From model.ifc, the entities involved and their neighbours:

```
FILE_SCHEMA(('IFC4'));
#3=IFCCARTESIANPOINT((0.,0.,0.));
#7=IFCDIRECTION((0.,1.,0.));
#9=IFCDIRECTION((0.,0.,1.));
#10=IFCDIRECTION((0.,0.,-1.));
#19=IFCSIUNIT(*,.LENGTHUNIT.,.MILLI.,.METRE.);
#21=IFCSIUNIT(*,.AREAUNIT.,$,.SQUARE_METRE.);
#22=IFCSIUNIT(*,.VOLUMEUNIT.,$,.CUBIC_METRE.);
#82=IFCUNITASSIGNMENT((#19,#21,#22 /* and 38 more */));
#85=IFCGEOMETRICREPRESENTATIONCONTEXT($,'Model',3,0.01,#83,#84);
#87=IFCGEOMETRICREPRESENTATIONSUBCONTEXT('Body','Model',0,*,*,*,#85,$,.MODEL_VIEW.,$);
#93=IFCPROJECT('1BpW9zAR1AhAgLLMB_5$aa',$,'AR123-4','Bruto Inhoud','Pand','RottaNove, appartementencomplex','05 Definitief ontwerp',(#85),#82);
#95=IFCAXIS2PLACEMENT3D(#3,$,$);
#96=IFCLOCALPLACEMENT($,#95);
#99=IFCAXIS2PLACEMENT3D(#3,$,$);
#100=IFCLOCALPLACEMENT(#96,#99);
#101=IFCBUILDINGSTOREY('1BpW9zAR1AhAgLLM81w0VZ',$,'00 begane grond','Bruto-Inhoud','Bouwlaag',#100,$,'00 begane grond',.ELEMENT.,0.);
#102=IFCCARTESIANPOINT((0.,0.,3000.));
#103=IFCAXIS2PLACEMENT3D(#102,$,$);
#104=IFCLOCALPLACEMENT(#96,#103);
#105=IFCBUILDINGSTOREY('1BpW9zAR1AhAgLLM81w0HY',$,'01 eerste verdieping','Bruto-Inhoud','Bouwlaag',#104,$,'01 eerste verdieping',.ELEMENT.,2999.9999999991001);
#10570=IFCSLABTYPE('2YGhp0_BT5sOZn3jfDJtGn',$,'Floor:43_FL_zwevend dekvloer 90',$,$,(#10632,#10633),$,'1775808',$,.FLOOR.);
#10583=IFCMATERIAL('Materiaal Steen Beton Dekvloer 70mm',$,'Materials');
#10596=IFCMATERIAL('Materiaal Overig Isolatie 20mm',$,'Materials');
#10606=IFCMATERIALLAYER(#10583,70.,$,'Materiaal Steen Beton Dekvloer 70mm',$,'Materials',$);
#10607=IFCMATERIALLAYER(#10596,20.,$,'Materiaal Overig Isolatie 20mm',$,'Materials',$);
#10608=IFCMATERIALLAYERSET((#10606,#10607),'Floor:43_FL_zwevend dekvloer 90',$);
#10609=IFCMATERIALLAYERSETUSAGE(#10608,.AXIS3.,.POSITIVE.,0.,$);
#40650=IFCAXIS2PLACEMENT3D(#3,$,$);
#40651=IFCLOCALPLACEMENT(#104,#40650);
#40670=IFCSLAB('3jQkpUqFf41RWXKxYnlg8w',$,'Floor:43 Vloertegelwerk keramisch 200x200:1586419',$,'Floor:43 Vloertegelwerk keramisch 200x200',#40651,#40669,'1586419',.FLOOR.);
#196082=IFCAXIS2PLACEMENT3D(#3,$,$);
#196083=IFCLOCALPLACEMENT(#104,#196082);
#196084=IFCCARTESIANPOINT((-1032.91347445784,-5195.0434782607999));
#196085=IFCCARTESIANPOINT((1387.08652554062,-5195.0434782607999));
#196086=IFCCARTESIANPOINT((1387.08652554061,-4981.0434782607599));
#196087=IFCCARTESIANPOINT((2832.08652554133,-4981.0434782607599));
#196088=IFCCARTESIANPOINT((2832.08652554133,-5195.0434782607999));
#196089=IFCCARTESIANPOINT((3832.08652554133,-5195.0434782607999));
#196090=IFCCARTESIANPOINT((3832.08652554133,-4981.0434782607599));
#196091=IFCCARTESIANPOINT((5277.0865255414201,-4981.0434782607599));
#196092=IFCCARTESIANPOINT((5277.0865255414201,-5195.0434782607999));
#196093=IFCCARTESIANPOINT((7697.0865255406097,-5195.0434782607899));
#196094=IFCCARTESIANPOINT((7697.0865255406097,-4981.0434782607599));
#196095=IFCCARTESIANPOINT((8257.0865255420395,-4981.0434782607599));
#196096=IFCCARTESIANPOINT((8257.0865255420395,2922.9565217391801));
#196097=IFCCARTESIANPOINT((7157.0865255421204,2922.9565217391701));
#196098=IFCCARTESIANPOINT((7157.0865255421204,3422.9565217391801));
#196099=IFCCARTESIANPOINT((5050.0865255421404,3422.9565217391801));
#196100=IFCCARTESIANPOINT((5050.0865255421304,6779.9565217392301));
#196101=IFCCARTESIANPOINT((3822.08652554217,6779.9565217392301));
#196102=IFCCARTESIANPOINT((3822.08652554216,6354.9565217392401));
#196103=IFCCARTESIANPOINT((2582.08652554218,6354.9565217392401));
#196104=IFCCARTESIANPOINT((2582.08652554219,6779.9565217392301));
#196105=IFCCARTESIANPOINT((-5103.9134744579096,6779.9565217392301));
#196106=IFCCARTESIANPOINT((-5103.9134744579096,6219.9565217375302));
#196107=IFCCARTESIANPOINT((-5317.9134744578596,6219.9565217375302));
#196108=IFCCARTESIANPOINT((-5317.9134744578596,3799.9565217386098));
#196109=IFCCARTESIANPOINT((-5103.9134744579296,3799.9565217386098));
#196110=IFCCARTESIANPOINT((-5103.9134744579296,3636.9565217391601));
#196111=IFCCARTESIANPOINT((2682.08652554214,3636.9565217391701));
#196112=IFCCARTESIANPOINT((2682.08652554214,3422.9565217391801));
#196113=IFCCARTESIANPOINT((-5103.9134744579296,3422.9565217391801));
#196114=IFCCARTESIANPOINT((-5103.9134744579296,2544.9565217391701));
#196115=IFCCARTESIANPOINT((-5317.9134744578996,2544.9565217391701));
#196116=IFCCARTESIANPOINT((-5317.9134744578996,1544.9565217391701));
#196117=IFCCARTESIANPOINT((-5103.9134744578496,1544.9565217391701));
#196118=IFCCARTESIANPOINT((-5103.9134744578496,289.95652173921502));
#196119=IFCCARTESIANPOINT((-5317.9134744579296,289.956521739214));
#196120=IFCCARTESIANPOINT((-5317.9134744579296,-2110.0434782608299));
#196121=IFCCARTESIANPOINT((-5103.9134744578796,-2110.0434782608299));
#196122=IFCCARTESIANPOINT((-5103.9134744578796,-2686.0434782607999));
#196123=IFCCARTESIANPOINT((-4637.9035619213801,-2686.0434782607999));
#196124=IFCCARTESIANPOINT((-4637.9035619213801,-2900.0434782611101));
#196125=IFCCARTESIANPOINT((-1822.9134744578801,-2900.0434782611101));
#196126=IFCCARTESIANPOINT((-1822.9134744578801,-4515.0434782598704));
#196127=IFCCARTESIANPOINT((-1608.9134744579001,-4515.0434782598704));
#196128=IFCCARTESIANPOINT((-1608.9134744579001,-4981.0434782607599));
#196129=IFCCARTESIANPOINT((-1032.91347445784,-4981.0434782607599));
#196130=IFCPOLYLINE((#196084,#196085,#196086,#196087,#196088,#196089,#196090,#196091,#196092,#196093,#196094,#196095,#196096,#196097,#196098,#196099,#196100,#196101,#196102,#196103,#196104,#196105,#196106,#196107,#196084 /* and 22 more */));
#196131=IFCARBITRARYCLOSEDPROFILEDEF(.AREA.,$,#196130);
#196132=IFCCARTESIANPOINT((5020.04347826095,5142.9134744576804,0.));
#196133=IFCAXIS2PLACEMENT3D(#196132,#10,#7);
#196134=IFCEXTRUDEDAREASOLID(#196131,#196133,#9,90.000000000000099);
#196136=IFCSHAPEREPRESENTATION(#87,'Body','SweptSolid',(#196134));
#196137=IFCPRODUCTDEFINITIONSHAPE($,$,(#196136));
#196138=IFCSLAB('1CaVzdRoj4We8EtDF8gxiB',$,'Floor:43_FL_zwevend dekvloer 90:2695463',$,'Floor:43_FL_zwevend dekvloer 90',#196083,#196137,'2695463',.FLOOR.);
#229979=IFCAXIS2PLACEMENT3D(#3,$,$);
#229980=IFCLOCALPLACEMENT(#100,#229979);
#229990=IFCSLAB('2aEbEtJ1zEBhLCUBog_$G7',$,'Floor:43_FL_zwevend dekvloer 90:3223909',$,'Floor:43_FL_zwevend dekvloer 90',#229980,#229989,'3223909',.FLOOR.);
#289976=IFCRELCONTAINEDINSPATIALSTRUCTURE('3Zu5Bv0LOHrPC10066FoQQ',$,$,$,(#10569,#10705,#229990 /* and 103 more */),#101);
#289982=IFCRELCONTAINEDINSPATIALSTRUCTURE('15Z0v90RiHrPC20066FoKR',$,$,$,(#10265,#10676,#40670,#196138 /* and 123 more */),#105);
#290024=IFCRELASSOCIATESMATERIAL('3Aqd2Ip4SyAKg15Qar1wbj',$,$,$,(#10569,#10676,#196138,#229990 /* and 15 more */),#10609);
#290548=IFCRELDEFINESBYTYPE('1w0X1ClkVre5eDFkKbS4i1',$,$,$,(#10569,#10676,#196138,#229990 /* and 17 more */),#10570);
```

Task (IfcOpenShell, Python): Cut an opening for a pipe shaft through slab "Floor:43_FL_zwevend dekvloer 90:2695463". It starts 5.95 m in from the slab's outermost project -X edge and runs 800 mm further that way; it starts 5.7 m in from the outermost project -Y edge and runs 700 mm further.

```python
import numpy as np
import ifcopenshell
import ifcopenshell.api.feature
import ifcopenshell.api.geometry
import ifcopenshell.api.root
import ifcopenshell.geom
import ifcopenshell.util.placement
import ifcopenshell.util.representation
import ifcopenshell.util.shape
import ifcopenshell.util.unit

model = ifcopenshell.open("model.ifc")
unit_scale = ifcopenshell.util.unit.calculate_unit_scale(model)
settings = ifcopenshell.geom.settings()


def volume(element):
    """Net volume in cubic metres, openings subtracted."""
    shape = ifcopenshell.geom.create_shape(settings, element)
    return ifcopenshell.util.shape.get_volume(shape.geometry)


slab = model.by_guid("1CaVzdRoj4We8EtDF8gxiB")
before = volume(slab)

# Extent in the slab's own axes, in metres. The edges named are its -X and -Y sides.
slab_shape = ifcopenshell.geom.create_shape(settings, slab)
vertices = ifcopenshell.util.shape.get_vertices(slab_shape.geometry)
x_min, y_min, bottom = vertices.min(axis=0)
top = vertices[:, 2].max()

opening = ifcopenshell.api.root.create_entity(model, ifc_class="IfcOpeningElement", name="Pipe shaft opening", predefined_type="OPENING")
context = ifcopenshell.util.representation.get_context(model, "Model", "Body", "MODEL_VIEW")
width, depth = 0.8, 0.7
outline = [(0.0, 0.0), (width, 0.0), (width, depth), (0.0, depth), (0.0, 0.0)]
# Overshoot both faces by 50 mm so the cut is clean.
shape = ifcopenshell.api.geometry.add_slab_representation(
    model, context=context, depth=top - bottom + 0.1, polyline=outline
)
ifcopenshell.api.geometry.assign_representation(model, product=opening, representation=shape)

matrix = ifcopenshell.util.placement.get_local_placement(slab.ObjectPlacement)
matrix[:, 3] = matrix @ np.append(np.array([x_min + 5.95, y_min + 5.7, bottom - 0.05]) / unit_scale, 1.0)
ifcopenshell.api.geometry.edit_object_placement(model, product=opening, matrix=matrix, is_si=False)
ifcopenshell.api.feature.add_feature(model, feature=opening, element=slab)

after = volume(slab)

print(f"slab volume {before:.3f} -> {after:.3f} m3")

model.write("model_edited.ifc")
```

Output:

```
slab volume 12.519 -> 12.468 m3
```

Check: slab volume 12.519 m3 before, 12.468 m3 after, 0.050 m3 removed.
